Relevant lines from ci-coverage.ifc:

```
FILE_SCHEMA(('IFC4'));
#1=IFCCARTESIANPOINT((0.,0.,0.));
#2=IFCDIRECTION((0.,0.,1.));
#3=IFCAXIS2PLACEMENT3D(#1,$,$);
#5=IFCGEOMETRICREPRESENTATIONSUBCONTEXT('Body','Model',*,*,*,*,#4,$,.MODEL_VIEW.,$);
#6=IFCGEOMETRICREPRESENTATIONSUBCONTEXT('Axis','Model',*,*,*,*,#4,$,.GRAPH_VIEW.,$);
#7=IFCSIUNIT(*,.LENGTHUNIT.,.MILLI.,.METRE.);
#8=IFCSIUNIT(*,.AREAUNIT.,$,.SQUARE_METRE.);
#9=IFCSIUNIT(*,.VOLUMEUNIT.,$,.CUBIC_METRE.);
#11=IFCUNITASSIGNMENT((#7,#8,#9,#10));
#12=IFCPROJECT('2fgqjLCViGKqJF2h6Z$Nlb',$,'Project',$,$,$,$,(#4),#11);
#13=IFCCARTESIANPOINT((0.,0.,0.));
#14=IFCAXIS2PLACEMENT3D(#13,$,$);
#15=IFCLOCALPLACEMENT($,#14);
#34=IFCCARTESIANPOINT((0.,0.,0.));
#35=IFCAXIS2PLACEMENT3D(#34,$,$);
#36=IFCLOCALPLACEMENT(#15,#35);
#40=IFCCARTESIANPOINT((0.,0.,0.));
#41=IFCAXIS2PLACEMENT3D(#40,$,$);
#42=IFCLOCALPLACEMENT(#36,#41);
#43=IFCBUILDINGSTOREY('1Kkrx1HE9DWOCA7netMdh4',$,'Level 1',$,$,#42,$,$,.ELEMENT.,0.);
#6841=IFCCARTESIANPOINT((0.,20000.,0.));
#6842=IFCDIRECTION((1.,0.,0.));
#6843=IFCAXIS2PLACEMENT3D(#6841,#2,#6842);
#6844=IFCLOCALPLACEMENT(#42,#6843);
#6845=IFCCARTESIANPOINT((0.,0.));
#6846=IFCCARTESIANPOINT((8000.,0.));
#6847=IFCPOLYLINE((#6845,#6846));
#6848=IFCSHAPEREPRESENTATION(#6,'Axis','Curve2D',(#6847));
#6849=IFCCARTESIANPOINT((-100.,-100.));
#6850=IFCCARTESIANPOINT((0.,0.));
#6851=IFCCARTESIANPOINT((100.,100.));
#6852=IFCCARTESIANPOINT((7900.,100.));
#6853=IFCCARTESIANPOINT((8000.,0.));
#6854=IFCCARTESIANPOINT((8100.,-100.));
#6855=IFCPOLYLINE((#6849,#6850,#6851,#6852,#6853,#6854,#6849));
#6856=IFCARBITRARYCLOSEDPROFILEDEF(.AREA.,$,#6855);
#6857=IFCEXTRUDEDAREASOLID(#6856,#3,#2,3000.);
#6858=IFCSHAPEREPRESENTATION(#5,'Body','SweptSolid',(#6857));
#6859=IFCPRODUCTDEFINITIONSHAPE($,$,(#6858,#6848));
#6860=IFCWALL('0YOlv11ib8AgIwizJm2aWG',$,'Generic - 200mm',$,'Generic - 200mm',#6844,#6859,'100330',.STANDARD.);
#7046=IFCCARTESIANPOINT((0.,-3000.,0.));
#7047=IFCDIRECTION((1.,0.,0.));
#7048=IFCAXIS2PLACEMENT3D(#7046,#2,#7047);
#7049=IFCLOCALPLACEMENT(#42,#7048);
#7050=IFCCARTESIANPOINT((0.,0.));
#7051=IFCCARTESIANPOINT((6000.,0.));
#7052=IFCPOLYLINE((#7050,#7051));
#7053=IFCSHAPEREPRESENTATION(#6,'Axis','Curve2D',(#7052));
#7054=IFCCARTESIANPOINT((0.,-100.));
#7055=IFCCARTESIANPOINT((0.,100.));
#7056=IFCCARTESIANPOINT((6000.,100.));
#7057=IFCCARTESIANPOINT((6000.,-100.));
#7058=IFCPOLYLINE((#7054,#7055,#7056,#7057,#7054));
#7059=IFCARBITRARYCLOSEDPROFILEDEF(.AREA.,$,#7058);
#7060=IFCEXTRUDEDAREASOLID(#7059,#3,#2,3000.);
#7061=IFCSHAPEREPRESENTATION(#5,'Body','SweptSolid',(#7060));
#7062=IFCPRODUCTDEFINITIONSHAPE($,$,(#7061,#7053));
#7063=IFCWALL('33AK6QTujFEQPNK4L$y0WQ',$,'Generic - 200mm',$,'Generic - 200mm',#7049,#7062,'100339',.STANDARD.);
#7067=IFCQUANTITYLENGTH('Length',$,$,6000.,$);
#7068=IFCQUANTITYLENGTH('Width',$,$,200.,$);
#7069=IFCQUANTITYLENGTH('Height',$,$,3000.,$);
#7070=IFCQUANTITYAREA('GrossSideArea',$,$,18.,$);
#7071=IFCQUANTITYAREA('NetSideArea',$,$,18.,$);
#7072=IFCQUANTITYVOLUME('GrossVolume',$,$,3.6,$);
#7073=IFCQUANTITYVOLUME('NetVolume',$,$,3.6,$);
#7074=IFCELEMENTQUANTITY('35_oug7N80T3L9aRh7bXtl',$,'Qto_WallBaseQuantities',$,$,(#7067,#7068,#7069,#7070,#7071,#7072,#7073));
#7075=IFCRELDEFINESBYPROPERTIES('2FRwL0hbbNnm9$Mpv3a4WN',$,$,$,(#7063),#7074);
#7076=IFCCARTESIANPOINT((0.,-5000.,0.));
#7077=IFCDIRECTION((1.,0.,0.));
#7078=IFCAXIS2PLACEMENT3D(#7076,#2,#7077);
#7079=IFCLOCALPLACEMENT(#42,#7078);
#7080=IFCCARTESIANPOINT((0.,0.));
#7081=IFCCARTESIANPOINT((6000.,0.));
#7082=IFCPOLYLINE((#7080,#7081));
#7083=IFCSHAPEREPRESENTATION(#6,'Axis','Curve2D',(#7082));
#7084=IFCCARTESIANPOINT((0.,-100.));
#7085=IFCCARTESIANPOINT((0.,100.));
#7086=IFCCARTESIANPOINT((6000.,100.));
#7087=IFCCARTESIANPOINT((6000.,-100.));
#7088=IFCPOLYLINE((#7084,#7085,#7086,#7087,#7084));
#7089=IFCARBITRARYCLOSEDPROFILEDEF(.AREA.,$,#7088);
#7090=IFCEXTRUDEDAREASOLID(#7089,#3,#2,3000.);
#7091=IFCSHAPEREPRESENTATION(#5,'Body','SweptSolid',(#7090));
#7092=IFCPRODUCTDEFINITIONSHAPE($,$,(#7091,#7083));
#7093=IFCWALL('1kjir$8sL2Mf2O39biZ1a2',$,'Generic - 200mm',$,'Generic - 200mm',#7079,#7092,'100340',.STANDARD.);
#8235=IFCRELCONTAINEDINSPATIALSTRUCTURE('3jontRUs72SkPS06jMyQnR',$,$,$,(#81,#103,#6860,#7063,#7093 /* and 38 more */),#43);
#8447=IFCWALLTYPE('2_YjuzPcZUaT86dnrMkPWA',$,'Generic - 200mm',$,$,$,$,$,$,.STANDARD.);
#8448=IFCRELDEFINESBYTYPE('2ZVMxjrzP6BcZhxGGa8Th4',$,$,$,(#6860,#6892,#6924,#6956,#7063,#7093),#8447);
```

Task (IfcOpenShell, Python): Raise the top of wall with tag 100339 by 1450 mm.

```python
import ifcopenshell
import ifcopenshell.api.pset
import ifcopenshell.geom
import ifcopenshell.util.element
import ifcopenshell.util.representation
import ifcopenshell.util.shape
import ifcopenshell.util.unit

model = ifcopenshell.open("ci-coverage.ifc")
unit_scale = ifcopenshell.util.unit.calculate_unit_scale(model)
area_scale = ifcopenshell.util.unit.calculate_unit_scale(model, "AREAUNIT")
volume_scale = ifcopenshell.util.unit.calculate_unit_scale(model, "VOLUMEUNIT")
settings = ifcopenshell.geom.settings()


def volume(element):
    """Net volume in cubic metres, openings subtracted."""
    shape = ifcopenshell.geom.create_shape(settings, element)
    return ifcopenshell.util.shape.get_volume(shape.geometry)


wall = model.by_guid("33AK6QTujFEQPNK4L$y0WQ")
before = volume(wall)

body = ifcopenshell.util.representation.get_representation(wall, "Model", "Body")
solid = body.Items[0]
old_height = solid.Depth
solid.Depth += 1.45 / unit_scale
after = volume(wall)
thickness = 0.2  # wall thickness in metres

# Update the stored height, areas and volumes.
qto = model.by_id(ifcopenshell.util.element.get_pset(wall, "Qto_WallBaseQuantities", should_inherit=False)["id"])
ifcopenshell.api.pset.edit_qto(model, qto=qto, properties={
    "Height": solid.Depth,
    "GrossSideArea": ifcopenshell.util.element.get_pset(wall, "Qto_WallBaseQuantities", "GrossSideArea") * solid.Depth / old_height,
    "NetSideArea": after / thickness / area_scale,
    "GrossVolume": ifcopenshell.util.element.get_pset(wall, "Qto_WallBaseQuantities", "GrossVolume") * solid.Depth / old_height,
    "NetVolume": after / volume_scale,
})

print(f"height {old_height:g} -> {solid.Depth:g}, volume {before:.3f} -> {after:.3f} m3")

model.write("ci-coverage_edited.ifc")
```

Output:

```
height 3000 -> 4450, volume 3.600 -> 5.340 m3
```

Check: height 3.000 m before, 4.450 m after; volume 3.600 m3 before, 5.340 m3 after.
